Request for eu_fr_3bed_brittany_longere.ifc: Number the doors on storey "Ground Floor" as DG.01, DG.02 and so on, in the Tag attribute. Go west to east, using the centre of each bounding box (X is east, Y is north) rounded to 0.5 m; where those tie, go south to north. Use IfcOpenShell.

First a look at what the model holds.

```python
import ifcopenshell
import ifcopenshell.util.element
import ifcopenshell.util.placement

model = ifcopenshell.open("eu_fr_3bed_brittany_longere.ifc")
print(model.schema)
storey = next(s for s in model.by_type("IfcBuildingStorey") if s.Name == "Ground Floor")
doors = [e for e in ifcopenshell.util.element.get_decomposition(storey) if e.is_a("IfcDoor")]
for e in sorted(doors, key=lambda e: e.id()):
    origin = ifcopenshell.util.placement.get_local_placement(e.ObjectPlacement)[:3, 3]
    print(e.id(), e.Tag, e.Name, origin.round(2) + 0.0, sep=" | ")
```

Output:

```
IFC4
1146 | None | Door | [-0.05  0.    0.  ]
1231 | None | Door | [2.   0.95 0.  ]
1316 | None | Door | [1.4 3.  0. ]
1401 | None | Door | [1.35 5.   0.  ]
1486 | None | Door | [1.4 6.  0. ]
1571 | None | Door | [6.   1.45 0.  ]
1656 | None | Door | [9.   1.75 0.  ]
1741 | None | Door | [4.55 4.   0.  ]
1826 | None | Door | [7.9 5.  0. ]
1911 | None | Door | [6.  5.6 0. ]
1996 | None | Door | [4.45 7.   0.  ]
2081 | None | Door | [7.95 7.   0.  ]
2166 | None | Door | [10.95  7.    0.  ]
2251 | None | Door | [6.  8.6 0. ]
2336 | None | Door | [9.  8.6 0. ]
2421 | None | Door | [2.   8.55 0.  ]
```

```python
import ifcopenshell
import ifcopenshell.geom
import ifcopenshell.util.element
import ifcopenshell.util.shape

model = ifcopenshell.open("eu_fr_3bed_brittany_longere.ifc")
settings = ifcopenshell.geom.settings()
settings.set("use-world-coords", True)


def centre(element):
    shape = ifcopenshell.geom.create_shape(settings, element)
    return ifcopenshell.util.shape.get_bbox_centroid(shape.geometry)


storey = next(s for s in model.by_type("IfcBuildingStorey") if s.Name == "Ground Floor")
doors = [e for e in ifcopenshell.util.element.get_decomposition(storey) if e.is_a("IfcDoor")]

# Insertion points can sit at a corner or the storey origin, so sort by the geometry (in metres).
centres = {e: centre(e) for e in doors}
doors.sort(key=lambda e: (round(centres[e][0] / 0.5), centres[e][1]))

for i, e in enumerate(doors, start=1):
    number = f"DG.{i:02d}"
    e.Tag = number
    print(e.id(), number)

model.write("eu_fr_3bed_brittany_longere_v2.ifc")
```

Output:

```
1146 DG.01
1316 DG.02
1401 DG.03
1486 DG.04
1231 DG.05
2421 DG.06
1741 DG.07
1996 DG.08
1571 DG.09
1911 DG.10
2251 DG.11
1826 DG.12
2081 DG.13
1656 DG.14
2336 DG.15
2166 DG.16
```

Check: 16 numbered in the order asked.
